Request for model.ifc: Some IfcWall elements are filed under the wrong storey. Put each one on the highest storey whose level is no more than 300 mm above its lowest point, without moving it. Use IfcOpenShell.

First a look at what the model holds.

```python
import ifcopenshell
import ifcopenshell.util.element
import ifcopenshell.util.placement

model = ifcopenshell.open("model.ifc")
print(model.schema)
for storey in model.by_type("IfcBuildingStorey"):
    level = ifcopenshell.util.placement.get_storey_elevation(storey)
    count = sum(e.is_a("IfcWall") for e in ifcopenshell.util.element.get_contained(storey))
    print(storey.id(), storey.Name, round(level, 3), count, sep=" | ")
```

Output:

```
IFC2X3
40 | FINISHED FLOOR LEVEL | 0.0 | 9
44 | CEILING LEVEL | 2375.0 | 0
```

```python
import ifcopenshell
import ifcopenshell.api.spatial
import ifcopenshell.geom
import ifcopenshell.util.element
import ifcopenshell.util.placement
import ifcopenshell.util.shape
import ifcopenshell.util.unit

model = ifcopenshell.open("model.ifc")
unit_scale = ifcopenshell.util.unit.calculate_unit_scale(model)
settings = ifcopenshell.geom.settings()

levels = sorted(
    ((ifcopenshell.util.placement.get_storey_elevation(s) * unit_scale, s) for s in model.by_type("IfcBuildingStorey")),
    key=lambda pair: pair[0],
)

for e in model.by_type("IfcWall"):
    current = e.ContainedInStructure[0].RelatingStructure if e.ContainedInStructure else None
    if current is None or not current.is_a("IfcBuildingStorey"):
        continue
    shape = ifcopenshell.geom.create_shape(settings, e)
    bottom = ifcopenshell.util.shape.get_shape_bottom_elevation(shape, shape.geometry)
    below = [s for level, s in levels if level <= bottom + 0.3]
    storey = below[-1] if below else levels[0][1]
    if storey != current:
        # assign_container keeps the world position.
        ifcopenshell.api.spatial.assign_container(model, products=[e], relating_structure=storey)
        print(e.id(), current.Name, "->", storey.Name)

model.write("model_rev.ifc")
```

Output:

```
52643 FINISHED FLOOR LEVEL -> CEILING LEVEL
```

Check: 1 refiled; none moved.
